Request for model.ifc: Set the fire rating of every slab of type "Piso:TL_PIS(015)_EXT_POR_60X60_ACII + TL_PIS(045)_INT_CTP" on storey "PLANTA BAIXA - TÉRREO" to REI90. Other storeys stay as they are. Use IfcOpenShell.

First a look at what the model holds.

```python
import ifcopenshell
import ifcopenshell.util.element

model = ifcopenshell.open("model.ifc")
print(model.schema)
storey = next(s for s in model.by_type("IfcBuildingStorey") if s.Name == "PLANTA BAIXA - TÉRREO")
slabs = [e for e in ifcopenshell.util.element.get_decomposition(storey) if e.is_a("IfcSlab")]
seen = {}
for e in slabs:
    element_type = ifcopenshell.util.element.get_type(e)
    key = (element_type.Name if element_type != e and element_type else None, ifcopenshell.util.element.get_pset(e, "Pset_SlabCommon", "FireRating"))
    seen[key] = seen.get(key, 0) + 1
for (name, value), count in sorted(seen.items(), key=str):
    print(count, "x", name, "|", value)
```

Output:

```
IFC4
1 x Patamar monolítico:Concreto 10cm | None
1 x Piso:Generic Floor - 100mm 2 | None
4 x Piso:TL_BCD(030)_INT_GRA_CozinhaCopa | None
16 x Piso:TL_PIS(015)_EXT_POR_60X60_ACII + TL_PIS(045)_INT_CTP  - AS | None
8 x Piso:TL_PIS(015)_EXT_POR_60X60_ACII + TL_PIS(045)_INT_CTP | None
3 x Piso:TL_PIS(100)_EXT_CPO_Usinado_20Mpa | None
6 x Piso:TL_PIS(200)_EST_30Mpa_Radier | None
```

```python
import ifcopenshell
import ifcopenshell.api.pset
import ifcopenshell.util.element

model = ifcopenshell.open("model.ifc")

storey = next(s for s in model.by_type("IfcBuildingStorey") if s.Name == "PLANTA BAIXA - TÉRREO")
slabs = [e for e in ifcopenshell.util.element.get_decomposition(storey) if e.is_a("IfcSlab")]

count = 0
for e in slabs:
    element_type = ifcopenshell.util.element.get_type(e)
    if element_type in (None, e) or element_type.Name != "Piso:TL_PIS(015)_EXT_POR_60X60_ACII + TL_PIS(045)_INT_CTP":
        continue
    # add_pset returns the element's existing set when there is one.
    pset = ifcopenshell.api.pset.add_pset(model, product=e, name="Pset_SlabCommon")
    ifcopenshell.api.pset.edit_pset(model, pset=pset, properties={"FireRating": "REI90"})
    count += 1

print(count, "slabs updated")

model.write("model-out.ifc")
```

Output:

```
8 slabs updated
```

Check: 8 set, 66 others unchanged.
